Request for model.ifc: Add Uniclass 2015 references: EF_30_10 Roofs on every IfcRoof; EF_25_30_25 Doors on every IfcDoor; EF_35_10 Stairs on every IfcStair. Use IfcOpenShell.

First a look at what the model holds.

```python
import ifcopenshell

model = ifcopenshell.open("model.ifc")
print(model.schema)
print("classifications:", [c.Name for c in model.by_type("IfcClassification")])
for ifc_class in ("IfcDoor", "IfcRoof", "IfcStair", "IfcWall", "IfcWindow"):
    print(ifc_class, len(model.by_type(ifc_class)))
```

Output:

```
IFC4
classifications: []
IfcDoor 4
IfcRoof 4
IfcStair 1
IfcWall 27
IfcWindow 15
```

```python
import ifcopenshell
import ifcopenshell.api.classification

model = ifcopenshell.open("model.ifc")

system = ifcopenshell.api.classification.add_classification(model, classification="Uniclass 2015")

codes = {
    "IfcRoof": ("EF_30_10", "Roofs"),
    "IfcDoor": ("EF_25_30_25", "Doors"),
    "IfcStair": ("EF_35_10", "Stairs"),
}
for ifc_class, (code, name) in codes.items():
    products = model.by_type(ifc_class)
    ifcopenshell.api.classification.add_reference(
        model, products=products, classification=system, identification=code, name=name
    )
    print(code, len(products))

model.write("model-out.ifc")
```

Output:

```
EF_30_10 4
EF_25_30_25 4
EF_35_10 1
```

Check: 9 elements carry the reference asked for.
